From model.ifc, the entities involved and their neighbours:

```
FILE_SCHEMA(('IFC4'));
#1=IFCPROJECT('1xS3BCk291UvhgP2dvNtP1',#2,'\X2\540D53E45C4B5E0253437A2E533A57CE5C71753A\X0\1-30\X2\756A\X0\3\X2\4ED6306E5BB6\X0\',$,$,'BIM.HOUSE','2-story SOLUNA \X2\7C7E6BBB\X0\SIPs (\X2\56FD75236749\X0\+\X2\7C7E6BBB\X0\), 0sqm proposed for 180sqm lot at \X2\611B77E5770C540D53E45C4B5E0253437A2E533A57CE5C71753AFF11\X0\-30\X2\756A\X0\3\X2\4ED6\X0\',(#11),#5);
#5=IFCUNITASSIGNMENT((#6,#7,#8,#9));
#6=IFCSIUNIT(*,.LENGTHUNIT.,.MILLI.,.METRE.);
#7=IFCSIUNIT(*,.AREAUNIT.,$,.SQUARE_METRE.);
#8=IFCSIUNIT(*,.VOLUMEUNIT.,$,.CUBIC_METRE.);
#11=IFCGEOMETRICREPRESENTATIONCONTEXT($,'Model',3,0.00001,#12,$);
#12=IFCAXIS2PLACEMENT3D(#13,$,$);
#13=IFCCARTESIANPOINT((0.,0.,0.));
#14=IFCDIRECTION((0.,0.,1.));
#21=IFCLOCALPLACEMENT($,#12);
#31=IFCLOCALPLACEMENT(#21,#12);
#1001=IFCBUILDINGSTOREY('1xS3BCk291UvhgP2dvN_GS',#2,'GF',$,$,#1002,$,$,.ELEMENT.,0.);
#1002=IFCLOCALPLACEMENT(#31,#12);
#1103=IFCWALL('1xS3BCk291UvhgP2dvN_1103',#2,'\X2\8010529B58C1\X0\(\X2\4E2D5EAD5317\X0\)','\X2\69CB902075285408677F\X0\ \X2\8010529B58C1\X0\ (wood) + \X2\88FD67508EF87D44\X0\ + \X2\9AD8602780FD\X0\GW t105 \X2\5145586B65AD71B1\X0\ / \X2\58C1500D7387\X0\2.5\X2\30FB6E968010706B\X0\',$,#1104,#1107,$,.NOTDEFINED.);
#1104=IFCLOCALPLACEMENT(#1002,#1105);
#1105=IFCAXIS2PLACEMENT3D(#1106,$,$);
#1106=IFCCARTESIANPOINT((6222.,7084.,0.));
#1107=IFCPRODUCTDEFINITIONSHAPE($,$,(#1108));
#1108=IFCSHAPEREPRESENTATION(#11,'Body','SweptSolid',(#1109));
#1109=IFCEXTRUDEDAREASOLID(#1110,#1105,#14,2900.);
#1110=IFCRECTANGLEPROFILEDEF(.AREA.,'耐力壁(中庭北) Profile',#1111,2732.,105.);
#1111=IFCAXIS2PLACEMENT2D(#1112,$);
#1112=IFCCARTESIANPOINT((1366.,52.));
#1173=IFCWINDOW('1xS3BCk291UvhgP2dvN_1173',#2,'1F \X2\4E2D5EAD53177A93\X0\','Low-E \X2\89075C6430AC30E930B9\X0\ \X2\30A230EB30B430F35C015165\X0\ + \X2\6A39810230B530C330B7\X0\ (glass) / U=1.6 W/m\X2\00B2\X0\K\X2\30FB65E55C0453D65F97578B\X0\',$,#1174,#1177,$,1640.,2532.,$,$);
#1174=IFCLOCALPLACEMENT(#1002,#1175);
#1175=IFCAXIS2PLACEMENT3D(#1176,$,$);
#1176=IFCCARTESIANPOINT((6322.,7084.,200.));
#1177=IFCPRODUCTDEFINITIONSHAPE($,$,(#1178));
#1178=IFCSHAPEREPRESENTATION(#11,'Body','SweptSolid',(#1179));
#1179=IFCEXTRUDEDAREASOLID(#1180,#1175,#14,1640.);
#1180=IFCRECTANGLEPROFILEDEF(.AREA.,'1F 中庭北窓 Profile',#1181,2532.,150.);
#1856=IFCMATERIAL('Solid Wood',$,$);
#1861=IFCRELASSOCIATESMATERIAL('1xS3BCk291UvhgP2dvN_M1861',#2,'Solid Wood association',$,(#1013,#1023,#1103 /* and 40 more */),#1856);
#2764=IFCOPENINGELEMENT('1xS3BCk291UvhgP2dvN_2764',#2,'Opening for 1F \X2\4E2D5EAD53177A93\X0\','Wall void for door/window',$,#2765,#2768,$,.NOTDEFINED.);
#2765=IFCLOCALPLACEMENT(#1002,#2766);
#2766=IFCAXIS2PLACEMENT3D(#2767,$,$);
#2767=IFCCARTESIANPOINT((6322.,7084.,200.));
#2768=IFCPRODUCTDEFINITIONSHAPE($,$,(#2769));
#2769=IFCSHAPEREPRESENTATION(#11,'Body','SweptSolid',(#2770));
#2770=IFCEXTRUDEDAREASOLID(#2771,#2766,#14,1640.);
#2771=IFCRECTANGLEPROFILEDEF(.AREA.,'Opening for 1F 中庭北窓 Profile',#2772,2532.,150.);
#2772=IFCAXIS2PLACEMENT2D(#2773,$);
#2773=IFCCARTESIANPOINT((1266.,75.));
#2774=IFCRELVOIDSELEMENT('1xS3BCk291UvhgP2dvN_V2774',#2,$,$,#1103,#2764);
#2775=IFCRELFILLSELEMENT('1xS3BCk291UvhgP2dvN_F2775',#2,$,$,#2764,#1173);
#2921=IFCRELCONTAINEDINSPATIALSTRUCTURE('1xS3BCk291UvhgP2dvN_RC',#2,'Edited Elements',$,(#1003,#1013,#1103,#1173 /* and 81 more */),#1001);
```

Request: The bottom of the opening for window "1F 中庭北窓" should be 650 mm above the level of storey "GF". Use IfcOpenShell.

```python
import numpy as np
import ifcopenshell
import ifcopenshell.api.geometry
import ifcopenshell.geom
import ifcopenshell.util.element
import ifcopenshell.util.placement
import ifcopenshell.util.shape
import ifcopenshell.util.unit

model = ifcopenshell.open("model.ifc")
unit_scale = ifcopenshell.util.unit.calculate_unit_scale(model)

window = model.by_guid("1xS3BCk291UvhgP2dvN_1173")
opening = window.FillsVoids[0].RelatingOpeningElement
storey = ifcopenshell.util.element.get_container(window, ifc_class="IfcBuildingStorey")
level = ifcopenshell.util.placement.get_local_placement(storey.ObjectPlacement)[2, 3]

# The opening's origin need not be at the sill, so measure its lowest point.
shape = ifcopenshell.geom.create_shape(ifcopenshell.geom.settings(), opening)
bottom = ifcopenshell.util.shape.get_shape_bottom_elevation(shape, shape.geometry) / unit_scale
dz = level + 650.0 - bottom

shift = np.array([0.0, 0.0, dz])
# The window is not placed relative to its opening, so move both.
for product in (opening, window):
    matrix = ifcopenshell.util.placement.get_local_placement(product.ObjectPlacement)
    matrix[:3, 3] += shift
    ifcopenshell.api.geometry.edit_object_placement(model, product=product, matrix=matrix, is_si=False)

print(f"moved by {dz * unit_scale:+.3f} m")

model.write("model_edited.ifc")
```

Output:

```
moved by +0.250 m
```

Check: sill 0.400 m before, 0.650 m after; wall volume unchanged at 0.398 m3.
